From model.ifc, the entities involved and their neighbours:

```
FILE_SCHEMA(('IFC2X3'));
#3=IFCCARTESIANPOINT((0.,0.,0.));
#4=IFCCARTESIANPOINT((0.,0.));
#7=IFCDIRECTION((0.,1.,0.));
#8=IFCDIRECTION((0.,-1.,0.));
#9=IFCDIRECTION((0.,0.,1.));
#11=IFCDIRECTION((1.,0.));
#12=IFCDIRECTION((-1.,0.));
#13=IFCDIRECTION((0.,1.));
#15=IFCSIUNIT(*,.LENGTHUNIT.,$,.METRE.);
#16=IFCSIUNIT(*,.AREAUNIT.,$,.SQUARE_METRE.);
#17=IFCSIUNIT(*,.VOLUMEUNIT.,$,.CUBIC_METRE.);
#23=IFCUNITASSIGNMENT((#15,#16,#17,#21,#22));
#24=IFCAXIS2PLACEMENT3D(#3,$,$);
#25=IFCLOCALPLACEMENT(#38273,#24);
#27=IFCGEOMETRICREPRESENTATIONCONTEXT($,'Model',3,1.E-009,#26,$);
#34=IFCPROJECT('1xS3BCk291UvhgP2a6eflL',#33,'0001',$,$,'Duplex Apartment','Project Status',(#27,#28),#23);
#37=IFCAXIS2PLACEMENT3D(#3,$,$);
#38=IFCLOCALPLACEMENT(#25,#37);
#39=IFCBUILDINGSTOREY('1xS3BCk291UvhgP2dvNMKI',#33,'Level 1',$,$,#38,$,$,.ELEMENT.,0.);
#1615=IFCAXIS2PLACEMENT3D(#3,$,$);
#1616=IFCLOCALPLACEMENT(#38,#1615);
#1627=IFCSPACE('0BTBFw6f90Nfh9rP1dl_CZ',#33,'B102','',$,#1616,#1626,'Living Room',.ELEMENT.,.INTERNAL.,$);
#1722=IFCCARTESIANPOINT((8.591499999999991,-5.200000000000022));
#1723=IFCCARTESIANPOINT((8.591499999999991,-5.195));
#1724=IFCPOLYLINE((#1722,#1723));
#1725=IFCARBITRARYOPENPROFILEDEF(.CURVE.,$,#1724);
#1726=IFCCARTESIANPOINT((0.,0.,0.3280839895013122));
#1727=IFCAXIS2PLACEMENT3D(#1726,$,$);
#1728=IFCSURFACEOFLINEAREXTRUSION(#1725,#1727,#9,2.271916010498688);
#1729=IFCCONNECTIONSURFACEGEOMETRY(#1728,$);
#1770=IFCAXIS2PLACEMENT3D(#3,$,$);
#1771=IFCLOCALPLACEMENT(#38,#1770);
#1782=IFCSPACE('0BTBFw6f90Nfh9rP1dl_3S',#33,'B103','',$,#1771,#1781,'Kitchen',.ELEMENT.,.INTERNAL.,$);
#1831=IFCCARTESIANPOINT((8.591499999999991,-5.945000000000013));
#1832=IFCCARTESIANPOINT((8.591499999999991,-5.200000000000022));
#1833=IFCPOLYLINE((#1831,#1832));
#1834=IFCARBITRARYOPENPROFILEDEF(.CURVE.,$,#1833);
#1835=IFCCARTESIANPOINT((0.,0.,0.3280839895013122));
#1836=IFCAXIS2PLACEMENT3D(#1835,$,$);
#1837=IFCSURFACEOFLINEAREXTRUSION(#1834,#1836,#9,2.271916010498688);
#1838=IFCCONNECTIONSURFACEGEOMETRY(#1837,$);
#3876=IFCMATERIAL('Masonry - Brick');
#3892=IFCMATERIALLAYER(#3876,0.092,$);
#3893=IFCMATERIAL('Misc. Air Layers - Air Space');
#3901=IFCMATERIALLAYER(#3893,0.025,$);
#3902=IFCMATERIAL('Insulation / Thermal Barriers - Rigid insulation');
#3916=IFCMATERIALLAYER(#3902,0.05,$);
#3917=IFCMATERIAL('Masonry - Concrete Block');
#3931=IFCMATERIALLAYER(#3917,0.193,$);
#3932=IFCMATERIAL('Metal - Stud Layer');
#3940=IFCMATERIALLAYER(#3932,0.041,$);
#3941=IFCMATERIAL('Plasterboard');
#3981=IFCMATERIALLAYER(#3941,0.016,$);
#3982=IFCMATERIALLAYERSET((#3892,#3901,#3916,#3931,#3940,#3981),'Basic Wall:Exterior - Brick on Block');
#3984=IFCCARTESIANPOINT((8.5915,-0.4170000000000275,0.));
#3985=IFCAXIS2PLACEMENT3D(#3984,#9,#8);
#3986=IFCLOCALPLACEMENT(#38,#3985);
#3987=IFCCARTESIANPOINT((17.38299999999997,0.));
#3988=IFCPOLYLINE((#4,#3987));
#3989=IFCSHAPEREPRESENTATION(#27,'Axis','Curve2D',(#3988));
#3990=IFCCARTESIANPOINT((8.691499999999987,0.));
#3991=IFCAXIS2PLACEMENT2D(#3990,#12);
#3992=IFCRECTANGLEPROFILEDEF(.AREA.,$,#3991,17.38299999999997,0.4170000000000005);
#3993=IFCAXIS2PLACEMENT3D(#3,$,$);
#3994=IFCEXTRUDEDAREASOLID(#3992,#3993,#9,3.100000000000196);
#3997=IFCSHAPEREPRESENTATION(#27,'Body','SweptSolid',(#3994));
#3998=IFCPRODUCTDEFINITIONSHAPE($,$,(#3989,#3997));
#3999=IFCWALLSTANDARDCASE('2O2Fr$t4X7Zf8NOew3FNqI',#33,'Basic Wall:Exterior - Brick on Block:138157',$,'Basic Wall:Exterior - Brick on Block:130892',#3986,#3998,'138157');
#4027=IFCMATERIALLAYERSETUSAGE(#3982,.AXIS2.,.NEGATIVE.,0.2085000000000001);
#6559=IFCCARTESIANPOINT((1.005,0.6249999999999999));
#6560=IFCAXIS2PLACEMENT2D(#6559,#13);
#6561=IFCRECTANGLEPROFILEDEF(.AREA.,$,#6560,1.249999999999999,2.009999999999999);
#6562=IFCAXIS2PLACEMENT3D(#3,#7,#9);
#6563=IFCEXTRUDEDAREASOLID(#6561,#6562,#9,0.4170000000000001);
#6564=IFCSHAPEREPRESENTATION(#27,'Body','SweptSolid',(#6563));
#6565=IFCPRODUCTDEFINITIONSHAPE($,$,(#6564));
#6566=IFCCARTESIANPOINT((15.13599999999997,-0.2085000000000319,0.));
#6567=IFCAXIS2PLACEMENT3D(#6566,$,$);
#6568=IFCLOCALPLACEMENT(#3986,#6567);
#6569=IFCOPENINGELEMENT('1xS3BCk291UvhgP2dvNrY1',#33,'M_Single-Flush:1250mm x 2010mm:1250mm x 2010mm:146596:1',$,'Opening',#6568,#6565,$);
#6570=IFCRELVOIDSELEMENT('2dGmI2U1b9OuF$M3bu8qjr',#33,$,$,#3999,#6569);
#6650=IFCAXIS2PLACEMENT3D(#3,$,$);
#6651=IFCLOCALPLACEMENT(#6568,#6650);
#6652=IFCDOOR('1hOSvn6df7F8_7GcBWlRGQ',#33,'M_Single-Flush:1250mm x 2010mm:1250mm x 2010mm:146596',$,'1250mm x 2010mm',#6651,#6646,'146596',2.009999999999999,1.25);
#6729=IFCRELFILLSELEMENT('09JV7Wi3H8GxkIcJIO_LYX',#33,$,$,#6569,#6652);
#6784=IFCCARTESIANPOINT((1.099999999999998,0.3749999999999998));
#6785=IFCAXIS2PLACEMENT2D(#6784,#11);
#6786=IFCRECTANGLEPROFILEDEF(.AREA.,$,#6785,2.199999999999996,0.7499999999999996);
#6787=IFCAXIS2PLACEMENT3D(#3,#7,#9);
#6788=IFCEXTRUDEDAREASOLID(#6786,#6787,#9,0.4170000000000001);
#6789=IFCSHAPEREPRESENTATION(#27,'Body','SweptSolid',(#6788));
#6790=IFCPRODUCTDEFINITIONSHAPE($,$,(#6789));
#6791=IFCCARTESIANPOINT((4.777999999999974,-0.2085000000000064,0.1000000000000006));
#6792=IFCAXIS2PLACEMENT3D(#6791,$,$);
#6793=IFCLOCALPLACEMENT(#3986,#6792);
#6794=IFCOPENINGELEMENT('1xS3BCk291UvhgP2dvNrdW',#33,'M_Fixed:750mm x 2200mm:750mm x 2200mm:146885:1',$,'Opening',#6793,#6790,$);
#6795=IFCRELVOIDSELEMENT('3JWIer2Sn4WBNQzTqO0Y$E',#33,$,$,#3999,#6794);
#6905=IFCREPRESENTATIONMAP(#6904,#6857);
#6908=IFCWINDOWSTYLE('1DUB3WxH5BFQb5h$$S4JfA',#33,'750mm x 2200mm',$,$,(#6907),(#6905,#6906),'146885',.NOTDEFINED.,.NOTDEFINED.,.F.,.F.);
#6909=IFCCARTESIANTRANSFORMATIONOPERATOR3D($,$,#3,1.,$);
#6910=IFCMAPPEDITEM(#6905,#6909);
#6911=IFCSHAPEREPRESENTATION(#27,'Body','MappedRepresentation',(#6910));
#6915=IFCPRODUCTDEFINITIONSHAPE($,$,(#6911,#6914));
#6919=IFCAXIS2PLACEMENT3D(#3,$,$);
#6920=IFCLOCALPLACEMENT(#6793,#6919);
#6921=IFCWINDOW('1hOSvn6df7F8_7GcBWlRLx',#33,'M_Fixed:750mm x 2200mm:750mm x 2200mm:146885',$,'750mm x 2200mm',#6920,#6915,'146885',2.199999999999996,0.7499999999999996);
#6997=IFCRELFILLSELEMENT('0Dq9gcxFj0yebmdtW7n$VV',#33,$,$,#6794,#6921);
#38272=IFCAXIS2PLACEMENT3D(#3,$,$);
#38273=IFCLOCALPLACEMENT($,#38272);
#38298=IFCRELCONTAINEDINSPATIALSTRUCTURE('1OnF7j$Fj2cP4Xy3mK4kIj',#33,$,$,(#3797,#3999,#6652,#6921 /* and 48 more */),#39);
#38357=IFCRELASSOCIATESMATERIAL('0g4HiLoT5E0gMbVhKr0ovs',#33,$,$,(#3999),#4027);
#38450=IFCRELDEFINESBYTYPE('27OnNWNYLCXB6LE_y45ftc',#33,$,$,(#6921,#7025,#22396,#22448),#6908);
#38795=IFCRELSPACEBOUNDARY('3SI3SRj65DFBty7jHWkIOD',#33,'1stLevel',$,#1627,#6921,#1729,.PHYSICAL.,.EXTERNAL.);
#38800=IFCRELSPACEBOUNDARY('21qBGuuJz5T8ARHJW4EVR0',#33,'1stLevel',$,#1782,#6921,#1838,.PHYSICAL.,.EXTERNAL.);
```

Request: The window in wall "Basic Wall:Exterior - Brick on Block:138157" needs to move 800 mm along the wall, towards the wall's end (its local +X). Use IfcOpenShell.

```python
import numpy as np
import ifcopenshell
import ifcopenshell.api.geometry
import ifcopenshell.util.placement
import ifcopenshell.util.unit

model = ifcopenshell.open("model.ifc")
unit_scale = ifcopenshell.util.unit.calculate_unit_scale(model)

window = model.by_guid("1hOSvn6df7F8_7GcBWlRLx")
opening = window.FillsVoids[0].RelatingOpeningElement
wall = opening.VoidsElements[0].RelatingBuildingElement

wall_matrix = ifcopenshell.util.placement.get_local_placement(wall.ObjectPlacement)
shift = wall_matrix[:3, 0] * 0.8 / unit_scale
before = ifcopenshell.util.placement.get_local_placement(window.ObjectPlacement)[:3, 3].copy()

# The window is placed relative to its opening, so it follows when the opening moves.
matrix = ifcopenshell.util.placement.get_local_placement(opening.ObjectPlacement)
matrix[:3, 3] += shift
ifcopenshell.api.geometry.edit_object_placement(
    model, product=opening, matrix=matrix, is_si=False, should_transform_children=True
)

# Space boundary surfaces are stored in each space's coordinates; move them too.
for rel in window.ProvidesBoundaries:
    if not rel.ConnectionGeometry:
        continue
    surface = rel.ConnectionGeometry.SurfaceOnRelatingElement
    space_matrix = ifcopenshell.util.placement.get_local_placement(rel.RelatingSpace.ObjectPlacement)
    point = np.array(surface.Position.Location.Coordinates) + space_matrix[:3, :3].T @ shift
    surface.Position = model.createIfcAxis2Placement3D(
        model.createIfcCartesianPoint(point.tolist()), surface.Position.Axis, surface.Position.RefDirection
    )

after = ifcopenshell.util.placement.get_local_placement(window.ObjectPlacement)[:3, 3]
print("window moved by", (after - before).round(3) + 0.0)

model.write("model_edited.ifc")
```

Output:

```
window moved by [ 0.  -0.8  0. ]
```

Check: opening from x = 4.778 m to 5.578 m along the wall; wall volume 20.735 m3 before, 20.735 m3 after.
